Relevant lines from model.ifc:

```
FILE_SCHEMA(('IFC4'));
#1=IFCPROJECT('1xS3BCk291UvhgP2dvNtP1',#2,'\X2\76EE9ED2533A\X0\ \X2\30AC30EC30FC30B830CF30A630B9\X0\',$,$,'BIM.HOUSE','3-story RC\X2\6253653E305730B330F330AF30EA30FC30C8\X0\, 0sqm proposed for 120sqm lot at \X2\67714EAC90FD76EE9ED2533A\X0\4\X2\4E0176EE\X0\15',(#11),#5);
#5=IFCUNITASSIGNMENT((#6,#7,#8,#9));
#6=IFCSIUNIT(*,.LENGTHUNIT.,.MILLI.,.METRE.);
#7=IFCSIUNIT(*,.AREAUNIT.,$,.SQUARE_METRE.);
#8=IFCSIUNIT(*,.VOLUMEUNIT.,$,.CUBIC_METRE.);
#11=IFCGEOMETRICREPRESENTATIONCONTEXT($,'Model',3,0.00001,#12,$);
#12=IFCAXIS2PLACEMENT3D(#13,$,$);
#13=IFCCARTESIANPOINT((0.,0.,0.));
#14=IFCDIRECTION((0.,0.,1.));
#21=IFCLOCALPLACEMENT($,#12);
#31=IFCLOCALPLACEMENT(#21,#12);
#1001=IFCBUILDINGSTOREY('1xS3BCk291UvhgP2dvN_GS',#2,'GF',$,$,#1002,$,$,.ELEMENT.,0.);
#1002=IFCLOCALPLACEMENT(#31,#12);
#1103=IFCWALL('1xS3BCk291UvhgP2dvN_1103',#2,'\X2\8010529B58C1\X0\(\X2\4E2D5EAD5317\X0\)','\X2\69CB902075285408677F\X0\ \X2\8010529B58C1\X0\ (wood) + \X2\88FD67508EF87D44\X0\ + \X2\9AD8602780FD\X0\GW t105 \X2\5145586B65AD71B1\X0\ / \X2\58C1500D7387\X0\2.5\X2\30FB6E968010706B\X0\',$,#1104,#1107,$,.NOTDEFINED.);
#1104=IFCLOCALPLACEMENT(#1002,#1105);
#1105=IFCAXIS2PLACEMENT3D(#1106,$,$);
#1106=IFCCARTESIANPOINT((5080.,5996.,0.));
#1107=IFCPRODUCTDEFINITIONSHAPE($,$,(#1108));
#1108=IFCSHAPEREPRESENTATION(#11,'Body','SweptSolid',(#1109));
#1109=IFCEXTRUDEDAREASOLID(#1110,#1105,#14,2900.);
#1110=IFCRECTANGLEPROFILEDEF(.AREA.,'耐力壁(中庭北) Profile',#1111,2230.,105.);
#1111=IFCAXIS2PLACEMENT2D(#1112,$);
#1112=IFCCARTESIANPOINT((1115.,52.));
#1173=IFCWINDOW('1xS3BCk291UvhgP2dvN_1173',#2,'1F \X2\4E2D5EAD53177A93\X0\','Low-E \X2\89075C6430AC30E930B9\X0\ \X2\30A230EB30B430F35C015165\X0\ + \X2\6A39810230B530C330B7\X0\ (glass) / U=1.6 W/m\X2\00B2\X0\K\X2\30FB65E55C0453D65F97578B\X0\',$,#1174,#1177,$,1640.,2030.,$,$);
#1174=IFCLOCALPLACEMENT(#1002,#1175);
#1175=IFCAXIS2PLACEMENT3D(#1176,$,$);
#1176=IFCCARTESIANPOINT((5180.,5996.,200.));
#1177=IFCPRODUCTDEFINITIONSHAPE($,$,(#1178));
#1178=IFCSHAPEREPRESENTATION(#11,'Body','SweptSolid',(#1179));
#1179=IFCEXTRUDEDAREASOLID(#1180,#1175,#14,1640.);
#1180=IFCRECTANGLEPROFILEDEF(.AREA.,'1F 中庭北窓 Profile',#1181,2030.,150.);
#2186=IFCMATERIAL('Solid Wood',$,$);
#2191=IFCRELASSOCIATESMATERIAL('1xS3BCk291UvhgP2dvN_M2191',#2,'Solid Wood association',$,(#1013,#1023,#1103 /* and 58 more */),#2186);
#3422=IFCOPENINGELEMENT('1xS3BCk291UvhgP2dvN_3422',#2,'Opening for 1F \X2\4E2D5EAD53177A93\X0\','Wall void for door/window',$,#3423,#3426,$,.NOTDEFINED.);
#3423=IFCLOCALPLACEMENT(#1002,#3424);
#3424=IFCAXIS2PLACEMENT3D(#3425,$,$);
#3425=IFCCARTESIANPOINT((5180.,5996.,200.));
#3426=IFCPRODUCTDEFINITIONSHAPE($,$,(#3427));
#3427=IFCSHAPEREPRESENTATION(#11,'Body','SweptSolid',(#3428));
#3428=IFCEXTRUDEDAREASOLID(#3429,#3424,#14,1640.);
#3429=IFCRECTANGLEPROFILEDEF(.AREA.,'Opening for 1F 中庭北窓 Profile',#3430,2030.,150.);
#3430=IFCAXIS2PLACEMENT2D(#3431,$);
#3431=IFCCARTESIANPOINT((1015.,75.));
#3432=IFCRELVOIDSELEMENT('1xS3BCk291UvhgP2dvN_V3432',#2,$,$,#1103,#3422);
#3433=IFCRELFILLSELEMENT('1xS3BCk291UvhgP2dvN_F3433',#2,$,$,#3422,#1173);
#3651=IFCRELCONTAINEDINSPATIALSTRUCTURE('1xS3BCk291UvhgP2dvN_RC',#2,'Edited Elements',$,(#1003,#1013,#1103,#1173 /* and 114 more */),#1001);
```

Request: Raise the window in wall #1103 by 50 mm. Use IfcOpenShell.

```python
import numpy as np
import ifcopenshell
import ifcopenshell.api.geometry
import ifcopenshell.util.placement
import ifcopenshell.util.unit

model = ifcopenshell.open("model.ifc")
unit_scale = ifcopenshell.util.unit.calculate_unit_scale(model)

window = model.by_guid("1xS3BCk291UvhgP2dvN_1173")
opening = window.FillsVoids[0].RelatingOpeningElement
dz = 0.05 / unit_scale

shift = np.array([0.0, 0.0, dz])
# The window is not placed relative to its opening, so move both.
for product in (opening, window):
    matrix = ifcopenshell.util.placement.get_local_placement(product.ObjectPlacement)
    matrix[:3, 3] += shift
    ifcopenshell.api.geometry.edit_object_placement(model, product=product, matrix=matrix, is_si=False)

print(f"moved by {dz * unit_scale:+.3f} m")

model.write("model_v2.ifc")
```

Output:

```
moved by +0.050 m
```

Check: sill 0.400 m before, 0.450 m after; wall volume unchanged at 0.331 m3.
